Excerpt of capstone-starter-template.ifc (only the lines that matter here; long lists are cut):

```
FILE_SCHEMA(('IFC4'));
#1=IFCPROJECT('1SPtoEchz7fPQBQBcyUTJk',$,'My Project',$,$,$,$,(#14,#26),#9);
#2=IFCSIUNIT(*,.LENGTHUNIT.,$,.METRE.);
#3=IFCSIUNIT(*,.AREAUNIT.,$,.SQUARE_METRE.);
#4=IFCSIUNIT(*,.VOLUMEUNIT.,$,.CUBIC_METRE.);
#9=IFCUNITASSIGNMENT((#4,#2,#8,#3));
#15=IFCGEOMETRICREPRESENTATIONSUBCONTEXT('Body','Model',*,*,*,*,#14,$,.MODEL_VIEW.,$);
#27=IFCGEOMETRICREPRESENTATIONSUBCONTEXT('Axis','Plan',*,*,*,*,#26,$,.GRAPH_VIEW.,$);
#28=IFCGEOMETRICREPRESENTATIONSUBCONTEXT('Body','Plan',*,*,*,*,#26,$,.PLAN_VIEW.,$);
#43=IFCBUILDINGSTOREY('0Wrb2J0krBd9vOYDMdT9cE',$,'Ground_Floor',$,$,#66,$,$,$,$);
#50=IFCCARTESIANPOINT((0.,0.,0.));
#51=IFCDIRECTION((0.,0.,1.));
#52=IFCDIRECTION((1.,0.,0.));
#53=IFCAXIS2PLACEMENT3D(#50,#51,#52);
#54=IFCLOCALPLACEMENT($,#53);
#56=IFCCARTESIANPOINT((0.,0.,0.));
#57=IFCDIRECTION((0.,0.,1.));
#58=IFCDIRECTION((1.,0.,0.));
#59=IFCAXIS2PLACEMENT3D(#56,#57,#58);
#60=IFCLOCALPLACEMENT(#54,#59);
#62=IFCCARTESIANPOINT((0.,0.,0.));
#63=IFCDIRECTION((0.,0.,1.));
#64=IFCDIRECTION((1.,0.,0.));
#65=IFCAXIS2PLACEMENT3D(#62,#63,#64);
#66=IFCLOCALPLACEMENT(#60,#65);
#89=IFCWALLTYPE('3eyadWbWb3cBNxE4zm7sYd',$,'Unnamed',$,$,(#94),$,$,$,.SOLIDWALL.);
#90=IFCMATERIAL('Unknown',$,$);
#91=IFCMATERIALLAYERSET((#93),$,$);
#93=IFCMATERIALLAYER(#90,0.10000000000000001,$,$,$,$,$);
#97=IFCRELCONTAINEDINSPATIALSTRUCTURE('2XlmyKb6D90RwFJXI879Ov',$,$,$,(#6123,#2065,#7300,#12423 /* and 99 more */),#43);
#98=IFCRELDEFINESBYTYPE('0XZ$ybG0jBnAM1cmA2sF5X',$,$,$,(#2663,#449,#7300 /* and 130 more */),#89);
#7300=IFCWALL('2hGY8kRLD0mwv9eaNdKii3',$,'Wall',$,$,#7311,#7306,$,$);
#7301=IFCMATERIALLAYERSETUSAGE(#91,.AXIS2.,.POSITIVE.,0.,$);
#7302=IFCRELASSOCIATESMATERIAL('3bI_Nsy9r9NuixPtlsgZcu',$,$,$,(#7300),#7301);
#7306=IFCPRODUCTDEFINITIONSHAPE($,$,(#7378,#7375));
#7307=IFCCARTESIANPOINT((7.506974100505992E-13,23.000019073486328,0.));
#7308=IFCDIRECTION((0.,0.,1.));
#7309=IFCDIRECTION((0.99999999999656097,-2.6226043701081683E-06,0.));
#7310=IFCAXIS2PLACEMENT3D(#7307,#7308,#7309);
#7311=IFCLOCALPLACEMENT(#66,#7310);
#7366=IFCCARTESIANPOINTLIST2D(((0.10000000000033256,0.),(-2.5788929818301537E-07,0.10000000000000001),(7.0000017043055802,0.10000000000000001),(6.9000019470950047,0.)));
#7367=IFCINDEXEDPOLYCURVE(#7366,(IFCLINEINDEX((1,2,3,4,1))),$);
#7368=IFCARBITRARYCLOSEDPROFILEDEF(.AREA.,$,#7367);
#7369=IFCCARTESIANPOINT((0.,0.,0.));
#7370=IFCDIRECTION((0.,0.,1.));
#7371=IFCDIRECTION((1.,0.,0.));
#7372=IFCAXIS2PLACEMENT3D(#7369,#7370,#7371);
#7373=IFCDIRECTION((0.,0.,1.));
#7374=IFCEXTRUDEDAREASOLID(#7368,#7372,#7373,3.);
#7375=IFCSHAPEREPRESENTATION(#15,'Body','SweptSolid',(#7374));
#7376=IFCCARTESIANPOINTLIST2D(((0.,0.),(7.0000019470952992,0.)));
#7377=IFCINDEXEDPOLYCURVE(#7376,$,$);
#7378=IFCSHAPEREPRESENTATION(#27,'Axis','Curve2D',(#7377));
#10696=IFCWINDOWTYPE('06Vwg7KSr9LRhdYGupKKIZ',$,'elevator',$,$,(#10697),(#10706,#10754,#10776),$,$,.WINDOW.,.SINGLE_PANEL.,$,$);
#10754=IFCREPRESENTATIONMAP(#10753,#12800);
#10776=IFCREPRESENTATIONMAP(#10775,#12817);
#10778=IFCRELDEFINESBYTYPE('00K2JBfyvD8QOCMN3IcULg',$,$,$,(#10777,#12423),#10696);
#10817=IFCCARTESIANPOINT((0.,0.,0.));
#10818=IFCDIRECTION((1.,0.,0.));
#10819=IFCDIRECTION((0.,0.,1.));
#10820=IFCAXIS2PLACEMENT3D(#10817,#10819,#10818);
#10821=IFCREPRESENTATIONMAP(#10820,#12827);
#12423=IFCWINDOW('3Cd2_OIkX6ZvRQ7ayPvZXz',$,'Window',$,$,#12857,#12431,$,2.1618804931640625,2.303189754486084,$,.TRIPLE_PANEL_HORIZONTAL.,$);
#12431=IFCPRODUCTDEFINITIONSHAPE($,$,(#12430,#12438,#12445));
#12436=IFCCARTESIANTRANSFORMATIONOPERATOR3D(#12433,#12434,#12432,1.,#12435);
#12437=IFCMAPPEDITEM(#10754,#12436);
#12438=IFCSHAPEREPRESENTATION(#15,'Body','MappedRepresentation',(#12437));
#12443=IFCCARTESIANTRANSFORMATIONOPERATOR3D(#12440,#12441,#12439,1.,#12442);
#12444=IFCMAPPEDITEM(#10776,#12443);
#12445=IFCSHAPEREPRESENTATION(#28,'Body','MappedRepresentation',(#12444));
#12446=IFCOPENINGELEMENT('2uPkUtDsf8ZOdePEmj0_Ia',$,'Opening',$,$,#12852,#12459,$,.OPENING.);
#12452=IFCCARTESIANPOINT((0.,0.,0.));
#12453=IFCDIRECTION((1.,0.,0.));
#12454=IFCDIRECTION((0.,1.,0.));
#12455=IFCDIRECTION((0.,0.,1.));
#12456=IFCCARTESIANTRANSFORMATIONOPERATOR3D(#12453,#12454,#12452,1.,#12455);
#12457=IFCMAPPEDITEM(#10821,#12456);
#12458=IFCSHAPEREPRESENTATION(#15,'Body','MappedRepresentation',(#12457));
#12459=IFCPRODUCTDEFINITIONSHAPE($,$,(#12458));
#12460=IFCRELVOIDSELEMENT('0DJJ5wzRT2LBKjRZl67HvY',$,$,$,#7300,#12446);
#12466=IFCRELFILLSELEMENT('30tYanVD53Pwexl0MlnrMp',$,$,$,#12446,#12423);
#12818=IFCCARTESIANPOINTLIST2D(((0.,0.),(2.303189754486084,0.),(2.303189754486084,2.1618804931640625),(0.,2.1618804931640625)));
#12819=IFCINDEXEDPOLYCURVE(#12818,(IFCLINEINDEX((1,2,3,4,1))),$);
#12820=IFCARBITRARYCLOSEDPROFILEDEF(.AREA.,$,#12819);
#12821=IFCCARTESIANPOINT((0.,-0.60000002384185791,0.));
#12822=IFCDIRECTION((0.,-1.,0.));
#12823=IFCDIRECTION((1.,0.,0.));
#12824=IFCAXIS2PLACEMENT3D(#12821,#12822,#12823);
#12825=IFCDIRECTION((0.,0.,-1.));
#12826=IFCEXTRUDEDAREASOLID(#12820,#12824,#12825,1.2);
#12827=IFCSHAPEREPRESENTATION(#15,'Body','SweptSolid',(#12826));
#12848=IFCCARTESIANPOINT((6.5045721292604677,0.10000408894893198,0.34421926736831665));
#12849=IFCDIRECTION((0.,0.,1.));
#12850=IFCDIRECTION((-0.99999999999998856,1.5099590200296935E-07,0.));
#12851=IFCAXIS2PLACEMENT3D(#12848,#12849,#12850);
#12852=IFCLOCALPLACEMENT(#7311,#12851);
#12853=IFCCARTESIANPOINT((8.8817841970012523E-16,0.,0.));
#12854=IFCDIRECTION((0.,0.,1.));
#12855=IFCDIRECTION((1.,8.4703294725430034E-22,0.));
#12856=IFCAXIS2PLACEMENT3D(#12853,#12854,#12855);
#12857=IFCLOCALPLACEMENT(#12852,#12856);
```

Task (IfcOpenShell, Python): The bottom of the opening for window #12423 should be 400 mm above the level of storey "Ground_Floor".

```python
import numpy as np
import ifcopenshell
import ifcopenshell.api.geometry
import ifcopenshell.geom
import ifcopenshell.util.element
import ifcopenshell.util.placement
import ifcopenshell.util.shape
import ifcopenshell.util.unit

model = ifcopenshell.open("capstone-starter-template.ifc")
unit_scale = ifcopenshell.util.unit.calculate_unit_scale(model)

window = model.by_id(12423)
opening = window.FillsVoids[0].RelatingOpeningElement
storey = ifcopenshell.util.element.get_container(window, ifc_class="IfcBuildingStorey")
level = ifcopenshell.util.placement.get_local_placement(storey.ObjectPlacement)[2, 3]

# The opening's origin need not be at the sill, so measure its lowest point.
shape = ifcopenshell.geom.create_shape(ifcopenshell.geom.settings(), opening)
bottom = ifcopenshell.util.shape.get_shape_bottom_elevation(shape, shape.geometry) / unit_scale
dz = level + 0.4 / unit_scale - bottom

shift = np.array([0.0, 0.0, dz])
# The window is placed relative to its opening, so it follows when the opening moves.
matrix = ifcopenshell.util.placement.get_local_placement(opening.ObjectPlacement)
matrix[:3, 3] += shift
ifcopenshell.api.geometry.edit_object_placement(
    model, product=opening, matrix=matrix, is_si=False, should_transform_children=True
)

print(f"moved by {dz * unit_scale:+.3f} m")

model.write("capstone-starter-template_rev.ifc")
```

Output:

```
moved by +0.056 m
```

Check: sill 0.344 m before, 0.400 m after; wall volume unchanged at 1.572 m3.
